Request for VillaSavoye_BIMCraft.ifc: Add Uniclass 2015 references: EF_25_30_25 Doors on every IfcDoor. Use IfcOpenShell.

First a look at what the model holds.

```python
import ifcopenshell

model = ifcopenshell.open("VillaSavoye_BIMCraft.ifc")
print(model.schema)
print("classifications:", [c.Name for c in model.by_type("IfcClassification")])
for ifc_class in ("IfcDoor", "IfcRoof", "IfcStair", "IfcWall", "IfcWindow"):
    print(ifc_class, len(model.by_type(ifc_class)))
```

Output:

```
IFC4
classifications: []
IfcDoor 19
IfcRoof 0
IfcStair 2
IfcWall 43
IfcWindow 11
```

```python
import ifcopenshell
import ifcopenshell.api.classification

model = ifcopenshell.open("VillaSavoye_BIMCraft.ifc")

system = ifcopenshell.api.classification.add_classification(model, classification="Uniclass 2015")

codes = {
    "IfcDoor": ("EF_25_30_25", "Doors"),
}
for ifc_class, (code, name) in codes.items():
    products = model.by_type(ifc_class)
    ifcopenshell.api.classification.add_reference(
        model, products=products, classification=system, identification=code, name=name
    )
    print(code, len(products))

model.write("VillaSavoye_BIMCraft_v2.ifc")
```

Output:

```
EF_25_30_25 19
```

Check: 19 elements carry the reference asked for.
